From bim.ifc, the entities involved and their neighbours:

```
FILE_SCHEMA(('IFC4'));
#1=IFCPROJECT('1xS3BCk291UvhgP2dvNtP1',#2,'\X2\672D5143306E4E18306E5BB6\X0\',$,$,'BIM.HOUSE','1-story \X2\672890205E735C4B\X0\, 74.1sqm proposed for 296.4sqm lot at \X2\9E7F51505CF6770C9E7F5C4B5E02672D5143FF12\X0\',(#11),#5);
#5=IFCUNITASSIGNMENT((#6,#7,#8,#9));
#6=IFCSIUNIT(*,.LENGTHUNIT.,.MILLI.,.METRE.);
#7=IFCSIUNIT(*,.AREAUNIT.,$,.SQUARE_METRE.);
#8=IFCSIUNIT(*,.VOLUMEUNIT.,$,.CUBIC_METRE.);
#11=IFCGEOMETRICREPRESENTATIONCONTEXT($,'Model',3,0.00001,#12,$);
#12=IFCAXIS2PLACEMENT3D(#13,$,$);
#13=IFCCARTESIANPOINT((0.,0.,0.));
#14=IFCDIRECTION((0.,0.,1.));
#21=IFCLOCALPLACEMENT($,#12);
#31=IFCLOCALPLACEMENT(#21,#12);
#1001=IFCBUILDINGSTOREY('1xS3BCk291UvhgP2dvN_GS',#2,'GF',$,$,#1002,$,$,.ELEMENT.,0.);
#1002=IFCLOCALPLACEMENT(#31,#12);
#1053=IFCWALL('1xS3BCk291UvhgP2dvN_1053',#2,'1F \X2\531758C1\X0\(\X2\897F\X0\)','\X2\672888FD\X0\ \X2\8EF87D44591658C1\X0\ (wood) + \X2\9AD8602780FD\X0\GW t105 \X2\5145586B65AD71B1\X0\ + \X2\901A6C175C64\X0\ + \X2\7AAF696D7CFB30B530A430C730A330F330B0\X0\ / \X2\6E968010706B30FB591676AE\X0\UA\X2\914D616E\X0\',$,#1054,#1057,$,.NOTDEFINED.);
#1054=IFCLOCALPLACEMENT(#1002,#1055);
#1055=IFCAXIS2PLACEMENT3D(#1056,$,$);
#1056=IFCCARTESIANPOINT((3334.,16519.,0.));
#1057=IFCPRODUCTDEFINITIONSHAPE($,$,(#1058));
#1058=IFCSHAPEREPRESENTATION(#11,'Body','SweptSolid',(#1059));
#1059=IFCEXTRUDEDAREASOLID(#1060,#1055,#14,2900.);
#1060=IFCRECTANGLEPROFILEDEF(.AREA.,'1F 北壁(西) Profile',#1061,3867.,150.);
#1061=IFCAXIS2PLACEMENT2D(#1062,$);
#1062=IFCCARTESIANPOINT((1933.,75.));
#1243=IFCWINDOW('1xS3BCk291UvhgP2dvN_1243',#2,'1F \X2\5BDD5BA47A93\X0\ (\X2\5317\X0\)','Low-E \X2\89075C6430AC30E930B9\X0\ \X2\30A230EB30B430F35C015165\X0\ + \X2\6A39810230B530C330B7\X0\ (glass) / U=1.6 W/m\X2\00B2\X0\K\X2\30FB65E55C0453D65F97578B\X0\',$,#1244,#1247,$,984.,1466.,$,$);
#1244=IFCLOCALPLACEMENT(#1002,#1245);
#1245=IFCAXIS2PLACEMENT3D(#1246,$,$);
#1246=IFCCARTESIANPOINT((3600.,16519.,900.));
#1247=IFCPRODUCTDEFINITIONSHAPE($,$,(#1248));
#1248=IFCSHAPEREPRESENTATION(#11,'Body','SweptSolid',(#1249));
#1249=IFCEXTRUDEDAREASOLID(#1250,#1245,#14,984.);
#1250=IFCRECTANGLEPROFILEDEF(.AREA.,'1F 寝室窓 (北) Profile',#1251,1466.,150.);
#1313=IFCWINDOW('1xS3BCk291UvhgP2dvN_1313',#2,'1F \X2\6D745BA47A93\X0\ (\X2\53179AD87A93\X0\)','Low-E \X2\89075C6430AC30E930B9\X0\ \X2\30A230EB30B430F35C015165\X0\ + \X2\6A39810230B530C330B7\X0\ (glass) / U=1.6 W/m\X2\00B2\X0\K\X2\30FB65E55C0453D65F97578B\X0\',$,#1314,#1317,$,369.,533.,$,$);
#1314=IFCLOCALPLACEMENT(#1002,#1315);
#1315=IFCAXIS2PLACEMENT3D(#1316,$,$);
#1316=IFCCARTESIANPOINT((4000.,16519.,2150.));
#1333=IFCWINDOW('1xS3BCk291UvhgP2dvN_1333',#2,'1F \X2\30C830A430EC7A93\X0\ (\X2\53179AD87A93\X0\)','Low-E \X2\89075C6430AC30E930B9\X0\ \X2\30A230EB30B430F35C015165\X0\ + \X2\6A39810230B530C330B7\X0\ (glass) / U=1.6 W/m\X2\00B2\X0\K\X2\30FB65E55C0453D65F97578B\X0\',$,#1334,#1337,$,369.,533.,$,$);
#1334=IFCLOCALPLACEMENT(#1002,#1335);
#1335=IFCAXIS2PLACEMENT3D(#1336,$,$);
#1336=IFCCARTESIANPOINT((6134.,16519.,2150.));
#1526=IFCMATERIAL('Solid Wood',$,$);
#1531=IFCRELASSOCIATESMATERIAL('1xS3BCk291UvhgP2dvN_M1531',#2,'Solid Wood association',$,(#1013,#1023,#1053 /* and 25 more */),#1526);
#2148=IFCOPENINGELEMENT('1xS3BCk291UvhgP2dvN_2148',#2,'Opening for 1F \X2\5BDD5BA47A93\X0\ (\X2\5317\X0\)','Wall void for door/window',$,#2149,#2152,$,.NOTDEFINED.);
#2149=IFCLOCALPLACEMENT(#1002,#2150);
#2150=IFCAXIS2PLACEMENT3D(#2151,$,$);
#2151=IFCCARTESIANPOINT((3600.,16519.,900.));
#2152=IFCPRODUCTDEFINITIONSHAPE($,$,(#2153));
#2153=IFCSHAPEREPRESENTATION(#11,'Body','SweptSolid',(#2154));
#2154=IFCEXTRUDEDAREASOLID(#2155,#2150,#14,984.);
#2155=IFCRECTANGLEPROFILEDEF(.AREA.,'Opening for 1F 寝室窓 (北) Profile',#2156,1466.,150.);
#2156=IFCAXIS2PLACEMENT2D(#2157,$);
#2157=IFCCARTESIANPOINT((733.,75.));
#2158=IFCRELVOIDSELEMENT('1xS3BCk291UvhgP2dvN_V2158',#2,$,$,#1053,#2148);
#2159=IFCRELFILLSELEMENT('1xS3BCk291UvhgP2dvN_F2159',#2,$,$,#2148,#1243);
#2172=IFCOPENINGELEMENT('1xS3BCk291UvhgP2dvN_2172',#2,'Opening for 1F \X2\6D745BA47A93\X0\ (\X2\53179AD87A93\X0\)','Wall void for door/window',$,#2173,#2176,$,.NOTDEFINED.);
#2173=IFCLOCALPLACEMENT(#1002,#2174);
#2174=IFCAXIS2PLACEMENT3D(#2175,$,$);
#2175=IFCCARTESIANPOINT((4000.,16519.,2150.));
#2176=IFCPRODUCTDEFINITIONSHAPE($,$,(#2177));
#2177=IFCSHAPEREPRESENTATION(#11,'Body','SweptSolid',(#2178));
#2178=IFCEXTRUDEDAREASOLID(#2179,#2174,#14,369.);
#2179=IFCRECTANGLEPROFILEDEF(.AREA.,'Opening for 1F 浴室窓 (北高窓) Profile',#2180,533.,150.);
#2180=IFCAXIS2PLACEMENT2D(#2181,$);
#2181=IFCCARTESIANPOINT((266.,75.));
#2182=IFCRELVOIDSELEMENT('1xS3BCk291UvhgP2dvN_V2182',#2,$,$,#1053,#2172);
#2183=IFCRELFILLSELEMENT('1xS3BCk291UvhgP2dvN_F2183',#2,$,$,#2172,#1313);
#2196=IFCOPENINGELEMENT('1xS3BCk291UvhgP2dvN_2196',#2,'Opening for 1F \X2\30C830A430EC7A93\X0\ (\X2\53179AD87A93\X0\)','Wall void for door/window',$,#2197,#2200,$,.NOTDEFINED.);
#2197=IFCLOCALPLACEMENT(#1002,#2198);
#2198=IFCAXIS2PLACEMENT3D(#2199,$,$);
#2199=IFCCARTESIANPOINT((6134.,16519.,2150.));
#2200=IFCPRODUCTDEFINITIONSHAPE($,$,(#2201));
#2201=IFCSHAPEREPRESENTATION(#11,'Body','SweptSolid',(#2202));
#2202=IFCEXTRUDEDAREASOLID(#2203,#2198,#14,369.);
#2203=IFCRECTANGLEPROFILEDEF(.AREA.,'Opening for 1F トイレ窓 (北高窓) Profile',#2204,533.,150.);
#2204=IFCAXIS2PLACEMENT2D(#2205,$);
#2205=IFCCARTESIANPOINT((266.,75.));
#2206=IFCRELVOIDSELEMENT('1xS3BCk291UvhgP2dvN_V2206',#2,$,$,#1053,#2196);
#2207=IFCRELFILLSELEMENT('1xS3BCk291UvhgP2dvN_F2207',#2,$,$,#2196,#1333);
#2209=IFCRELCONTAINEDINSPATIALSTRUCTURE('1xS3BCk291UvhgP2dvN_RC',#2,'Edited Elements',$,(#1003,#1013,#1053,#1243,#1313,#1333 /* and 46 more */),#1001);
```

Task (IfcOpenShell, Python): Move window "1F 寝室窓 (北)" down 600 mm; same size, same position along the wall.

```python
import numpy as np
import ifcopenshell
import ifcopenshell.api.geometry
import ifcopenshell.util.placement
import ifcopenshell.util.unit

model = ifcopenshell.open("bim.ifc")
unit_scale = ifcopenshell.util.unit.calculate_unit_scale(model)

window = model.by_id(1243)
opening = window.FillsVoids[0].RelatingOpeningElement
dz = -600.0

shift = np.array([0.0, 0.0, dz])
# The window is not placed relative to its opening, so move both.
for product in (opening, window):
    matrix = ifcopenshell.util.placement.get_local_placement(product.ObjectPlacement)
    matrix[:3, 3] += shift
    ifcopenshell.api.geometry.edit_object_placement(model, product=product, matrix=matrix, is_si=False)

print(f"moved by {dz * unit_scale:+.3f} m")

model.write("bim_updated.ifc")
```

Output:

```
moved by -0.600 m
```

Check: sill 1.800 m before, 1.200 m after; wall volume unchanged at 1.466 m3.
